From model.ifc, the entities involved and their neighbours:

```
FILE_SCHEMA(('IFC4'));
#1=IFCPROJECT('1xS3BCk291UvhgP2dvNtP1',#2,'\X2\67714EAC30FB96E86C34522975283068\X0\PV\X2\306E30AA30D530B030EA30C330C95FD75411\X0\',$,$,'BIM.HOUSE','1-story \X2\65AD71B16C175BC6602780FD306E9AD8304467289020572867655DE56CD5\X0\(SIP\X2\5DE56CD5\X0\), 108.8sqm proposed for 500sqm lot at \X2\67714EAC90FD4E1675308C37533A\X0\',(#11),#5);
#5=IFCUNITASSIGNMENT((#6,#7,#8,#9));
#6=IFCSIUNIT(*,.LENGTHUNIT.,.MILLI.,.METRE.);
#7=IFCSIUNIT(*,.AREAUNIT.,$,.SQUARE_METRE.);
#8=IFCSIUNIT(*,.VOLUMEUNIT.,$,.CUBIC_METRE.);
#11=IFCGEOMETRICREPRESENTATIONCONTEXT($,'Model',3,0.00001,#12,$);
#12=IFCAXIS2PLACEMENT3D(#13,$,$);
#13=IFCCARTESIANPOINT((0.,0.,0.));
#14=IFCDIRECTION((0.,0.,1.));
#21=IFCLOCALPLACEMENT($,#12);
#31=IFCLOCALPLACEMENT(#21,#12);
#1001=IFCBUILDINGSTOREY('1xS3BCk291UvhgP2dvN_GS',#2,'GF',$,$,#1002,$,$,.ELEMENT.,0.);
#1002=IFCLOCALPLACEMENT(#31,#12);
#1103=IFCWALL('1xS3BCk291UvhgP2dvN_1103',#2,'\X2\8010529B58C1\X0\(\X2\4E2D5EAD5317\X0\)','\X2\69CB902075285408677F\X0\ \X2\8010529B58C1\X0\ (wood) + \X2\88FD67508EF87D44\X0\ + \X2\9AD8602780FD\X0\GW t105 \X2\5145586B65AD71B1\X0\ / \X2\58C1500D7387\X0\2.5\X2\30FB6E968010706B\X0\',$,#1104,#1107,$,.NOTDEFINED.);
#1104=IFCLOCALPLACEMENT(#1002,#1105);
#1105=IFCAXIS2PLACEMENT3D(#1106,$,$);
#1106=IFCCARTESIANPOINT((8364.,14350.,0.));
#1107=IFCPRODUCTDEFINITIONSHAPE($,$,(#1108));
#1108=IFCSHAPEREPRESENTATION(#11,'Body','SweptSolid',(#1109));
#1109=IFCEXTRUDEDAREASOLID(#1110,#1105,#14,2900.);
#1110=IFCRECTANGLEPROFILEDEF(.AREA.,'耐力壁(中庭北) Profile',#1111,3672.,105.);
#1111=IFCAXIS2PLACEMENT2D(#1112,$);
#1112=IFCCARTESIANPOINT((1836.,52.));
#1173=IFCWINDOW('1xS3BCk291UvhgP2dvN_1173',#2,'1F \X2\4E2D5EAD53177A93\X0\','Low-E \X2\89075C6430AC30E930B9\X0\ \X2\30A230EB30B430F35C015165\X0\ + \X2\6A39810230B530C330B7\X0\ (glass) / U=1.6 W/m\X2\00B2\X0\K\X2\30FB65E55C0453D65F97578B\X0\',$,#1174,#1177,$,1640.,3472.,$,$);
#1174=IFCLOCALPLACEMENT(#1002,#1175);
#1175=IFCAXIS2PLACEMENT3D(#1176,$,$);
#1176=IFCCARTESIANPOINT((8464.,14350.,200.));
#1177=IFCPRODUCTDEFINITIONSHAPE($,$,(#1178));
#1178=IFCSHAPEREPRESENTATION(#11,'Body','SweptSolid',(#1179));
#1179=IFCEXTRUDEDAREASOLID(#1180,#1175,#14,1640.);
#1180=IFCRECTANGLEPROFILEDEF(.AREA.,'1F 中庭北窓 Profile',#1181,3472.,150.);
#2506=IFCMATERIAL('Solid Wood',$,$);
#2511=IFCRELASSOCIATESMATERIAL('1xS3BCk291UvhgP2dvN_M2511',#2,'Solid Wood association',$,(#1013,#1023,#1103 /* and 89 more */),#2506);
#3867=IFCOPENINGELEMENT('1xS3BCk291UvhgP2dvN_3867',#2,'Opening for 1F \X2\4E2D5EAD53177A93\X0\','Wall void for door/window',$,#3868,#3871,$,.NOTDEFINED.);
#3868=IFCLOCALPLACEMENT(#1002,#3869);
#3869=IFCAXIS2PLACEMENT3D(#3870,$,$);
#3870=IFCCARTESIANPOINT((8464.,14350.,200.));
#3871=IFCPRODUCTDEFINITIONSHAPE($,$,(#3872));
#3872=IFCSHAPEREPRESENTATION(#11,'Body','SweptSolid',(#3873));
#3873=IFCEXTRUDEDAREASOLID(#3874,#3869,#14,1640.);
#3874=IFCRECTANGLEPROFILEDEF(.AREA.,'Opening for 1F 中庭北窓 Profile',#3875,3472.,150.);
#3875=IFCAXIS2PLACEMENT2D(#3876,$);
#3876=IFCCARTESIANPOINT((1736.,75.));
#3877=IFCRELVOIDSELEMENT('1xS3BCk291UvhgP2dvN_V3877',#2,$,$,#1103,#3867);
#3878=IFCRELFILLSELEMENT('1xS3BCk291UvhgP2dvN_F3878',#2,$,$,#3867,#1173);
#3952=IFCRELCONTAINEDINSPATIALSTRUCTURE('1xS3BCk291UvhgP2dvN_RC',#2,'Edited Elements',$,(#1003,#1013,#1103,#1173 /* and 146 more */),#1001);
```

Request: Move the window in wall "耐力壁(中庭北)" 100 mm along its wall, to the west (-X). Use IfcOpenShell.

```python
import ifcopenshell
import ifcopenshell.api.geometry
import ifcopenshell.util.placement
import ifcopenshell.util.unit

model = ifcopenshell.open("model.ifc")
unit_scale = ifcopenshell.util.unit.calculate_unit_scale(model)

window = model.by_guid("1xS3BCk291UvhgP2dvN_1173")
opening = window.FillsVoids[0].RelatingOpeningElement
wall = opening.VoidsElements[0].RelatingBuildingElement

wall_matrix = ifcopenshell.util.placement.get_local_placement(wall.ObjectPlacement)
shift = wall_matrix[:3, 0] * -0.1 / unit_scale
before = ifcopenshell.util.placement.get_local_placement(window.ObjectPlacement)[:3, 3].copy()

# The window is not placed relative to its opening, so move both.
for product in (opening, window):
    matrix = ifcopenshell.util.placement.get_local_placement(product.ObjectPlacement)
    matrix[:3, 3] += shift
    ifcopenshell.api.geometry.edit_object_placement(model, product=product, matrix=matrix, is_si=False)

after = ifcopenshell.util.placement.get_local_placement(window.ObjectPlacement)[:3, 3]
print("window moved by", (after - before).round(3) + 0.0)

model.write("model-out.ifc")
```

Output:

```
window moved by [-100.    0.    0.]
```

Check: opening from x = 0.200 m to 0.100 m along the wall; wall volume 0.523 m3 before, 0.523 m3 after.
